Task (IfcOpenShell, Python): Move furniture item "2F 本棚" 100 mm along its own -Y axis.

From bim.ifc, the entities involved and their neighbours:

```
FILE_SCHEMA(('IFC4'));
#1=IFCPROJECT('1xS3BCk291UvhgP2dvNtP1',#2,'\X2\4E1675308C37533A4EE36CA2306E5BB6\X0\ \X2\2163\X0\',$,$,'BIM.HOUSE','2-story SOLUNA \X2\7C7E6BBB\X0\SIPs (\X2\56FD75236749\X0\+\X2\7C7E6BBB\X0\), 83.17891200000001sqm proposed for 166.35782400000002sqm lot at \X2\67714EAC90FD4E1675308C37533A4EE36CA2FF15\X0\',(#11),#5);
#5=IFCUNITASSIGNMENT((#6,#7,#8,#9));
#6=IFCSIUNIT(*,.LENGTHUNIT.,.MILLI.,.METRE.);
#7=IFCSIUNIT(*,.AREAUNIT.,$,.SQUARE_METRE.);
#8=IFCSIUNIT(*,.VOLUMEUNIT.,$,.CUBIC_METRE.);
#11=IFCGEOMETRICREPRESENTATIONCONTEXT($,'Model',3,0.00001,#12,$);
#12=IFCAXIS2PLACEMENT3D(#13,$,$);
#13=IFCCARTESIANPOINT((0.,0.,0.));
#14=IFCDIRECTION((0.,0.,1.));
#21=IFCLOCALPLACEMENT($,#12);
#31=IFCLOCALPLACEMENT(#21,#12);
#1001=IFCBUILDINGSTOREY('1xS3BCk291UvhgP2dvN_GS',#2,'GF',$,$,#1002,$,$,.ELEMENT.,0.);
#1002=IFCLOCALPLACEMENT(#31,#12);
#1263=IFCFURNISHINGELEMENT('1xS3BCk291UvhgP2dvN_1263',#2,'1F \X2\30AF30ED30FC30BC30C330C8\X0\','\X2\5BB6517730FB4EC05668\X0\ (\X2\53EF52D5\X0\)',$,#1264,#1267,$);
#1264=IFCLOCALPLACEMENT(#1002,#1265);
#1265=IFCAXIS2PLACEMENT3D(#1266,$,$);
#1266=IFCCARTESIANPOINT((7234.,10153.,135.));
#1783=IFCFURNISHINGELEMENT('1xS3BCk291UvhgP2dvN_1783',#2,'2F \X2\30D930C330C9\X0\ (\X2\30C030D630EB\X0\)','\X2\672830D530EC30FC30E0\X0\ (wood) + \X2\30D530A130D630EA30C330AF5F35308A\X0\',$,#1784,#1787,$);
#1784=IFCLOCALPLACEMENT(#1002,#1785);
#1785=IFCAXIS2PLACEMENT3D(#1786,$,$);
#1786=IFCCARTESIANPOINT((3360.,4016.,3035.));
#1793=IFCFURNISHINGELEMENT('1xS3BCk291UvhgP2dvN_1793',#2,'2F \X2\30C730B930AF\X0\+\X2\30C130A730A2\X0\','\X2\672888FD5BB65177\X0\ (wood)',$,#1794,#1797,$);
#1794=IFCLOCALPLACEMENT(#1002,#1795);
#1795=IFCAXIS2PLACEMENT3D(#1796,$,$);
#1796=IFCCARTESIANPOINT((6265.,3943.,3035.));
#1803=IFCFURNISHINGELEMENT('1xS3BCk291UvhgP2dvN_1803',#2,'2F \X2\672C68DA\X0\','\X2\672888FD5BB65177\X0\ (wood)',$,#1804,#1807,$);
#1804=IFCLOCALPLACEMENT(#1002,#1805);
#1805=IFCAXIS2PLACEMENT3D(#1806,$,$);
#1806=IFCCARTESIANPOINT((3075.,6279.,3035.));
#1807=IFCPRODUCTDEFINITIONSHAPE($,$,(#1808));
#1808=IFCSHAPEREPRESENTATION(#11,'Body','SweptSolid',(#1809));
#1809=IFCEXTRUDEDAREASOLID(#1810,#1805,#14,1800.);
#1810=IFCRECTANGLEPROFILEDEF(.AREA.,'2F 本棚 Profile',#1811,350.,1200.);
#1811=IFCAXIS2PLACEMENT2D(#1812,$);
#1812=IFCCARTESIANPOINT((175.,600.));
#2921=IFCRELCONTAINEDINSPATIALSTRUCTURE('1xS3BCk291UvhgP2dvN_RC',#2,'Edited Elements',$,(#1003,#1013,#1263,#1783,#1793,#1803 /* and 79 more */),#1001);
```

```python
import ifcopenshell
import ifcopenshell.api.geometry
import ifcopenshell.util.placement

model = ifcopenshell.open("bim.ifc")

item = model.by_guid("1xS3BCk291UvhgP2dvN_1803")
matrix = ifcopenshell.util.placement.get_local_placement(item.ObjectPlacement)
matrix[:3, 3] -= matrix[:3, 1] * 100.0
ifcopenshell.api.geometry.edit_object_placement(model, product=item, matrix=matrix, is_si=False)

print(ifcopenshell.util.placement.get_local_placement(item.ObjectPlacement).round(3) + 0.0)

model.write("bim_rev.ifc")
```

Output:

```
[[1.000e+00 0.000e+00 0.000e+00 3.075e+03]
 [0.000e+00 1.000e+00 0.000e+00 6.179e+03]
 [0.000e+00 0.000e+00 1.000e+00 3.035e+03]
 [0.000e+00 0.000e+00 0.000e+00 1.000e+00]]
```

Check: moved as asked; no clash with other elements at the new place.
